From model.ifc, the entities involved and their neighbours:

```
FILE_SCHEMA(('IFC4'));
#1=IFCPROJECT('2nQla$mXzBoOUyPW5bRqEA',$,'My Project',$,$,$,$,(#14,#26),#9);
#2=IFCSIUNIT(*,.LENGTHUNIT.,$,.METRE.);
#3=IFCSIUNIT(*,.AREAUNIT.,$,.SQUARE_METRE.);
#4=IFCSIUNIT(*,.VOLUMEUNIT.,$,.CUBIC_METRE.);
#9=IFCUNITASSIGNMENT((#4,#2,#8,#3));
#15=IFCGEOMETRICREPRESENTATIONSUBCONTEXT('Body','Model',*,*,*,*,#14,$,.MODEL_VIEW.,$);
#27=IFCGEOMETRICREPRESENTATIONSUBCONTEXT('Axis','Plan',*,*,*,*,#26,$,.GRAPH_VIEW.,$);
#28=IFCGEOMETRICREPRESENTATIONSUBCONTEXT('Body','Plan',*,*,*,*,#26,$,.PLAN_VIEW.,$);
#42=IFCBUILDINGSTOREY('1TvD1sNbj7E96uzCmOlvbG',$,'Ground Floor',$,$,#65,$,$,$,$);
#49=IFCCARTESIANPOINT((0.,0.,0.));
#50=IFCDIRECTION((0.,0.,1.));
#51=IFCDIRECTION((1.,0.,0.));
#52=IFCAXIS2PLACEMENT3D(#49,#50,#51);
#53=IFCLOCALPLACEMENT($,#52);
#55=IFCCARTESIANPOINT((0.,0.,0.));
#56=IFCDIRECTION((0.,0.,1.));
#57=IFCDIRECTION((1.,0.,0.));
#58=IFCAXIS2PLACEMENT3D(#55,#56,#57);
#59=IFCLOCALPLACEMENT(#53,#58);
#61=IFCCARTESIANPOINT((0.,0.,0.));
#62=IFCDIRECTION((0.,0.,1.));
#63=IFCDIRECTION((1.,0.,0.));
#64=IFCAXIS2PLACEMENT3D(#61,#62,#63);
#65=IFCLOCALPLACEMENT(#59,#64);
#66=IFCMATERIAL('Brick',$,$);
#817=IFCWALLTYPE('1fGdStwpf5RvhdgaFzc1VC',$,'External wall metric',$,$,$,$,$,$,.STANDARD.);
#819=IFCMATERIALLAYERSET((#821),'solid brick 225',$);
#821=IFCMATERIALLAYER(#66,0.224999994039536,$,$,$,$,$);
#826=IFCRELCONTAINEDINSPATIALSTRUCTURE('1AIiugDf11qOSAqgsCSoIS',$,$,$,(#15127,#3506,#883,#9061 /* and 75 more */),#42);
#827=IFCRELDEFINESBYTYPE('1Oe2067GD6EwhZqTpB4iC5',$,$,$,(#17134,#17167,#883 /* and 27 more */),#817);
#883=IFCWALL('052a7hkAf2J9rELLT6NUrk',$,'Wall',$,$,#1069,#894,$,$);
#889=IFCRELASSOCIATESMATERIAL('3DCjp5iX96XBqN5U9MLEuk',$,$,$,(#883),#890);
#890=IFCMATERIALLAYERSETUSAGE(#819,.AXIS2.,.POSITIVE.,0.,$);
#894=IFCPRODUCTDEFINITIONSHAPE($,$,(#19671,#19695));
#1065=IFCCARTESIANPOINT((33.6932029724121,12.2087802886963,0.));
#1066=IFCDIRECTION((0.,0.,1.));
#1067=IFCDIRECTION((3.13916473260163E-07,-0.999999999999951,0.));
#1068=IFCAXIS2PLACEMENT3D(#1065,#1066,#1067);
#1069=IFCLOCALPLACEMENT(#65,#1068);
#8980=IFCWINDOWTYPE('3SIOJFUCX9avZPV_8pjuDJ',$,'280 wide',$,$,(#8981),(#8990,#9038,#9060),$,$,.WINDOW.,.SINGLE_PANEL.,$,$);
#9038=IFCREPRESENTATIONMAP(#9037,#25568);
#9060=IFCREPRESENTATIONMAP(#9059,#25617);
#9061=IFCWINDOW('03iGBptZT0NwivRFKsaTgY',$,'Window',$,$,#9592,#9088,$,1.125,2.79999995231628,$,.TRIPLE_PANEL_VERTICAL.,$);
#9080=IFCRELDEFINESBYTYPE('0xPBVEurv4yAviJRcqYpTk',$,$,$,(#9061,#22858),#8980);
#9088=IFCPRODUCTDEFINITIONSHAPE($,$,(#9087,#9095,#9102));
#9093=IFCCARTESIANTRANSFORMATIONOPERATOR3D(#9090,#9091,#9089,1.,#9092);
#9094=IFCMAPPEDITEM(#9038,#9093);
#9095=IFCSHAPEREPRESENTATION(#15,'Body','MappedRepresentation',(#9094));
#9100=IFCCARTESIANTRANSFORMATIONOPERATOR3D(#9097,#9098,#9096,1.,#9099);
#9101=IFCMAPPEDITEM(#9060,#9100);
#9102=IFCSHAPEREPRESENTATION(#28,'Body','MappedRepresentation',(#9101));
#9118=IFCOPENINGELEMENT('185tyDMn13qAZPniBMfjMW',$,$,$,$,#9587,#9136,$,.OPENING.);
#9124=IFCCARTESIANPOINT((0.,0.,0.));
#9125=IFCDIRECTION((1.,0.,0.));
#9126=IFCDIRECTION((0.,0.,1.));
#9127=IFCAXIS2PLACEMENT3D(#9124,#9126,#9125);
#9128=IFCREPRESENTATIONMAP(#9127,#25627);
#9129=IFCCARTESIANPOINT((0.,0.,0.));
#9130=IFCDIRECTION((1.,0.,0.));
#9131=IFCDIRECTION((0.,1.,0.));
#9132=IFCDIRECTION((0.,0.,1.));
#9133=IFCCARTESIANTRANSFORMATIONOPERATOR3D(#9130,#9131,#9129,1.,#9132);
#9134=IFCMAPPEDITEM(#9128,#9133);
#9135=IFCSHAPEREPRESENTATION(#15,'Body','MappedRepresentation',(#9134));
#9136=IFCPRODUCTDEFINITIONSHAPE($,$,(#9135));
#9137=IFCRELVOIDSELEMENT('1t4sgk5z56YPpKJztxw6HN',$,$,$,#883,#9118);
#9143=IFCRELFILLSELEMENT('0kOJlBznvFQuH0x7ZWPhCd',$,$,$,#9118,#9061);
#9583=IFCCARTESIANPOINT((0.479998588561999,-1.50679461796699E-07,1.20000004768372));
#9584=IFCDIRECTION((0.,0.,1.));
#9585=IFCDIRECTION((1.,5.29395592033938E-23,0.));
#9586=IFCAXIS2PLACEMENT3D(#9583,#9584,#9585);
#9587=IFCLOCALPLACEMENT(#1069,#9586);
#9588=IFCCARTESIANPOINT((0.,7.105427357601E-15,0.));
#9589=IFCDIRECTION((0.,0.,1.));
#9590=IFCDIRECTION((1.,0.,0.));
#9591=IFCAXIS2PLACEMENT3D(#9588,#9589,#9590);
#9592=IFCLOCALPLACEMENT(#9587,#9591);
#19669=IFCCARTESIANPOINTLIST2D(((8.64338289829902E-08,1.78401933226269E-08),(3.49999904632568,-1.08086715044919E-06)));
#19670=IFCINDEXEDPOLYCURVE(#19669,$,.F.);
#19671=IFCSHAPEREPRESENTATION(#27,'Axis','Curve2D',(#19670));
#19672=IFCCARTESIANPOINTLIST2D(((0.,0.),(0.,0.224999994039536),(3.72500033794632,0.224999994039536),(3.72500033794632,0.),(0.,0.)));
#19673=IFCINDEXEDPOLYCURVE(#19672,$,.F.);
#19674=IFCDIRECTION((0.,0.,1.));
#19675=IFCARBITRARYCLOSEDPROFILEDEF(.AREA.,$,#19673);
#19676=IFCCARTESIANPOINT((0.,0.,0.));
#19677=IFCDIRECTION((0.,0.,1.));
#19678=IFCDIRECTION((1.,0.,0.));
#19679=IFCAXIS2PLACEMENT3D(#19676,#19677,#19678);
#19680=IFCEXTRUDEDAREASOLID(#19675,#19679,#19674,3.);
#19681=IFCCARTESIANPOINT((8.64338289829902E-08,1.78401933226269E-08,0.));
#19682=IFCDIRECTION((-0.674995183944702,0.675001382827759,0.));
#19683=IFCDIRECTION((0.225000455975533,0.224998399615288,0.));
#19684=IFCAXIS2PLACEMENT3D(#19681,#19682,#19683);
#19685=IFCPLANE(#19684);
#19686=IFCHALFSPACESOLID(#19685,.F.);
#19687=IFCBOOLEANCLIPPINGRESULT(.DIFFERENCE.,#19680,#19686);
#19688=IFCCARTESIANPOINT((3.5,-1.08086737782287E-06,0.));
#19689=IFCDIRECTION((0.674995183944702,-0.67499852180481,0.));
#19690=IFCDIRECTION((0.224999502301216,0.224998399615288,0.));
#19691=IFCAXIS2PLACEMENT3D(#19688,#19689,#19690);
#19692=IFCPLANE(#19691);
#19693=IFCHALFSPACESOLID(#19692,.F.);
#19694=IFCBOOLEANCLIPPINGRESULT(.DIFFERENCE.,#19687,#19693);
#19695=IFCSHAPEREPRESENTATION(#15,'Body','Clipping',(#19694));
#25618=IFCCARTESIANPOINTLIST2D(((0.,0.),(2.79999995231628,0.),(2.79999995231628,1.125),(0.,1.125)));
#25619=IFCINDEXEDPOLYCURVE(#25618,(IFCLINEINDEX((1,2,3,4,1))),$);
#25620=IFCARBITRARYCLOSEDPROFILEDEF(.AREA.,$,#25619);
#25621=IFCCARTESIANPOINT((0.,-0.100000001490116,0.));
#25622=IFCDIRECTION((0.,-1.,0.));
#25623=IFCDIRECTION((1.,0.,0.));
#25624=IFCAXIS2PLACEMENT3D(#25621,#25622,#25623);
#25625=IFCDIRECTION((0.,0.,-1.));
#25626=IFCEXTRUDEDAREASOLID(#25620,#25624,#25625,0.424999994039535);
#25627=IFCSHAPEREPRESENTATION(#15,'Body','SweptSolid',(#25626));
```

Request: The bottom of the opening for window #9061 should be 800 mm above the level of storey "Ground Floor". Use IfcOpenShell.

```python
import numpy as np
import ifcopenshell
import ifcopenshell.api.geometry
import ifcopenshell.geom
import ifcopenshell.util.element
import ifcopenshell.util.placement
import ifcopenshell.util.shape
import ifcopenshell.util.unit

model = ifcopenshell.open("model.ifc")
unit_scale = ifcopenshell.util.unit.calculate_unit_scale(model)

window = model.by_guid("03iGBptZT0NwivRFKsaTgY")
opening = window.FillsVoids[0].RelatingOpeningElement
storey = ifcopenshell.util.element.get_container(window, ifc_class="IfcBuildingStorey")
level = ifcopenshell.util.placement.get_local_placement(storey.ObjectPlacement)[2, 3]

# The opening's origin need not be at the sill, so measure its lowest point.
shape = ifcopenshell.geom.create_shape(ifcopenshell.geom.settings(), opening)
bottom = ifcopenshell.util.shape.get_shape_bottom_elevation(shape, shape.geometry) / unit_scale
dz = level + 0.8 - bottom

shift = np.array([0.0, 0.0, dz])
# The window is placed relative to its opening, so it follows when the opening moves.
matrix = ifcopenshell.util.placement.get_local_placement(opening.ObjectPlacement)
matrix[:3, 3] += shift
ifcopenshell.api.geometry.edit_object_placement(
    model, product=opening, matrix=matrix, is_si=False, should_transform_children=True
)

print(f"moved by {dz * unit_scale:+.3f} m")

model.write("model_updated.ifc")
```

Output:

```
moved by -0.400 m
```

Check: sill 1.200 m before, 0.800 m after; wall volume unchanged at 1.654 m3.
